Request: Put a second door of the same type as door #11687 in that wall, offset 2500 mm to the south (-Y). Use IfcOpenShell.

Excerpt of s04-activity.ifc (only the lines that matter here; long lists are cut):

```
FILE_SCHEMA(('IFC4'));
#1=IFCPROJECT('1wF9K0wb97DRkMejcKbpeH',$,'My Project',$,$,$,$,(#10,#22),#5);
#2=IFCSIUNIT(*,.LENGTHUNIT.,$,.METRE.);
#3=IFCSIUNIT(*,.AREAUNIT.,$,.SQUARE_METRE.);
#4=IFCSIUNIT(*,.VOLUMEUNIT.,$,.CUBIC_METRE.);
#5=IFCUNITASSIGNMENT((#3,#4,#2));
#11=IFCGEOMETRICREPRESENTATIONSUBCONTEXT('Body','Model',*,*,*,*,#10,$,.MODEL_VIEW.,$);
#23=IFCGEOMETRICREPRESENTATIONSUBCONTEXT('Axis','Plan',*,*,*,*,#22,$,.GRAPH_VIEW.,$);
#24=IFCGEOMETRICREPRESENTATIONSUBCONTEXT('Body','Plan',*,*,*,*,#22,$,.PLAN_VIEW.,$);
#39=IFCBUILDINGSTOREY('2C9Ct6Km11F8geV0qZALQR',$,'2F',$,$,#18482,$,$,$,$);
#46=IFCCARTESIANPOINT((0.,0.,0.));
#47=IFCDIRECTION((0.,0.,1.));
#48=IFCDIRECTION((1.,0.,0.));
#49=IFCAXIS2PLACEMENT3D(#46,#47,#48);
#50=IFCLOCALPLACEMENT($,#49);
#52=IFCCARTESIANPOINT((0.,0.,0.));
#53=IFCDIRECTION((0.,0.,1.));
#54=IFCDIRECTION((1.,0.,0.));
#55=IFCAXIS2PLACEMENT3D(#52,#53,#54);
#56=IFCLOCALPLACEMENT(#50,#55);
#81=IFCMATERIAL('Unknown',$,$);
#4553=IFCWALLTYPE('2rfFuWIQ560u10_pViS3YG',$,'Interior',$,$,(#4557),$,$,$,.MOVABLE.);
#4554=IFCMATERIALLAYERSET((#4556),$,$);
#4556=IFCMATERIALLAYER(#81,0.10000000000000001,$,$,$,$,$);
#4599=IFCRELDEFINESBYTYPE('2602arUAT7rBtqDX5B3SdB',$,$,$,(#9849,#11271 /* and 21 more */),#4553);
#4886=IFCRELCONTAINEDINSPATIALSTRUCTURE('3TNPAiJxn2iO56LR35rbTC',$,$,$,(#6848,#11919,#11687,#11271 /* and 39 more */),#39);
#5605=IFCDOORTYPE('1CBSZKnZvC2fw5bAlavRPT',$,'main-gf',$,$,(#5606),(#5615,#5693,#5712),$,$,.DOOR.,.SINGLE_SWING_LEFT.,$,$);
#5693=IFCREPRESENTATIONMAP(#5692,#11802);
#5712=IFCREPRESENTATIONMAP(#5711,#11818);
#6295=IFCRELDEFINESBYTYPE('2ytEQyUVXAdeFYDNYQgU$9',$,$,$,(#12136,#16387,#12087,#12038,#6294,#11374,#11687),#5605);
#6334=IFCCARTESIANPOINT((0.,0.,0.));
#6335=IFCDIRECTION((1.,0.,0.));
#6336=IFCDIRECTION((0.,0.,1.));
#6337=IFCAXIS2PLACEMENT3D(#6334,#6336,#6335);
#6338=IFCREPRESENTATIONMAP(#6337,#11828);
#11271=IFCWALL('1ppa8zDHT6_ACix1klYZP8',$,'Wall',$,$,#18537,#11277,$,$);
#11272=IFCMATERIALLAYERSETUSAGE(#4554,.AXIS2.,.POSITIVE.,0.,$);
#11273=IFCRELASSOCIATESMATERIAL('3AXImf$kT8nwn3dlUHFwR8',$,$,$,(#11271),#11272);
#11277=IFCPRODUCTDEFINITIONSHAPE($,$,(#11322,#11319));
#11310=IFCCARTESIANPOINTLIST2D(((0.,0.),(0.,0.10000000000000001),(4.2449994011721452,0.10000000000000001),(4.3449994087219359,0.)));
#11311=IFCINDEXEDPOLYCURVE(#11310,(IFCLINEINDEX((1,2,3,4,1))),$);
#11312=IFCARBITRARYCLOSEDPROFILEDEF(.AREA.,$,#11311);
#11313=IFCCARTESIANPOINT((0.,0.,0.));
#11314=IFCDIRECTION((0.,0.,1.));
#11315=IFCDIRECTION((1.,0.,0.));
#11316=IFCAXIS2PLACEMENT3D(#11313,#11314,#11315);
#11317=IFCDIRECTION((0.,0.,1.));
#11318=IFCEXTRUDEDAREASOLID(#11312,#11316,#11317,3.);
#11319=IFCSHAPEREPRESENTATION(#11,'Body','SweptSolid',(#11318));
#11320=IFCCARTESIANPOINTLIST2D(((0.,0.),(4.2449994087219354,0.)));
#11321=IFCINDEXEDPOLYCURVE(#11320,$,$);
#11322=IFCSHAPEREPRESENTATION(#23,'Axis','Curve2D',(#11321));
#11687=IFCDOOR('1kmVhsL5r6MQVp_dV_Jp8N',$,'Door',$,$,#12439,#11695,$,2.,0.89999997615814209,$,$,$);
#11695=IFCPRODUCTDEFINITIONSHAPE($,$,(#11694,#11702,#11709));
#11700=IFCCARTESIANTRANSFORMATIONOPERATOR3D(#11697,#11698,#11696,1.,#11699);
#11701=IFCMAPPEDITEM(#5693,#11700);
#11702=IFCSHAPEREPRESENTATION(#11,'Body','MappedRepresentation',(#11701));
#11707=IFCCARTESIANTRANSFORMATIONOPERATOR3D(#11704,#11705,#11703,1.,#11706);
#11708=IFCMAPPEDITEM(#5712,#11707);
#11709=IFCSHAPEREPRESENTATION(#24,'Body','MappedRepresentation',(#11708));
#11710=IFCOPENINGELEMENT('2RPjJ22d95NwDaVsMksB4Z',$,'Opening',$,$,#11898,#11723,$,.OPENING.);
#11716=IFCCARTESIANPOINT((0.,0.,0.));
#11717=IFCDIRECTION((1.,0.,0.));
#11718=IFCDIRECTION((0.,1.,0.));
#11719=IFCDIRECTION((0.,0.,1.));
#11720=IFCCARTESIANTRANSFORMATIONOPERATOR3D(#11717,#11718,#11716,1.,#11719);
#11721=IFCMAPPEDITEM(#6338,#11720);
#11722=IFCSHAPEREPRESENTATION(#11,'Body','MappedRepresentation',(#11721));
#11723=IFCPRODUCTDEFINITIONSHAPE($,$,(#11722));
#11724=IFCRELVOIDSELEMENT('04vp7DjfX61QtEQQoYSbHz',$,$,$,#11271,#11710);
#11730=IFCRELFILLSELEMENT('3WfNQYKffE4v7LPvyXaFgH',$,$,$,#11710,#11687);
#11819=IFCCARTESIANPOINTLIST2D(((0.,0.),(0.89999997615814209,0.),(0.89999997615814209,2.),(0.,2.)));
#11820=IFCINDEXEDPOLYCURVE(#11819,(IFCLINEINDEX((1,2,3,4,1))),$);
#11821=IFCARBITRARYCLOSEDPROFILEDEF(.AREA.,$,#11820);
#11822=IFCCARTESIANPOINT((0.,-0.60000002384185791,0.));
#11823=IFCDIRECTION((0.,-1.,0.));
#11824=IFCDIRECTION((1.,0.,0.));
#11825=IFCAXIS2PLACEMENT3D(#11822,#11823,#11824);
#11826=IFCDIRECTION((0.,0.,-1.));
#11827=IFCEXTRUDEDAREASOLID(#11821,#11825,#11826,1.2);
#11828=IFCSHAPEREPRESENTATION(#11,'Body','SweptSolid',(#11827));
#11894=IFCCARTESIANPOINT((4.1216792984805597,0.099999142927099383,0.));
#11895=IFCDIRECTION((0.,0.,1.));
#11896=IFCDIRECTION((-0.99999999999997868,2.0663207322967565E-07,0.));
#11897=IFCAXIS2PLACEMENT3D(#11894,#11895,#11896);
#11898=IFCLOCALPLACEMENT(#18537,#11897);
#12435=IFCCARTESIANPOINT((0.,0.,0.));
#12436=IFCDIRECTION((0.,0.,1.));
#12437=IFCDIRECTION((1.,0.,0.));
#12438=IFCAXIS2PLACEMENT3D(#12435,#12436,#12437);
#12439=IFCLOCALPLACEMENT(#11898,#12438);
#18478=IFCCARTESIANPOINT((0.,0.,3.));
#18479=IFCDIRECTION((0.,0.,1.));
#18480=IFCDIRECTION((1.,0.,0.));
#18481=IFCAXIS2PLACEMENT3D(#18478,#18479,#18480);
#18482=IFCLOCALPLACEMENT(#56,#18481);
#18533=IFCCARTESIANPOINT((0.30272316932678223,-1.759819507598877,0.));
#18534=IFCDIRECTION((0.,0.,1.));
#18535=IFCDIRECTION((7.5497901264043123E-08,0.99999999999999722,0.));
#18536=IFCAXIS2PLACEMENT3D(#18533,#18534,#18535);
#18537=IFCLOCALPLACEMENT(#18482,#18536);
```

```python
import ifcopenshell
import ifcopenshell.api.feature
import ifcopenshell.api.geometry
import ifcopenshell.api.root
import ifcopenshell.geom
import ifcopenshell.util.element
import ifcopenshell.util.placement
import ifcopenshell.util.shape
import ifcopenshell.util.unit

model = ifcopenshell.open("s04-activity.ifc")
unit_scale = ifcopenshell.util.unit.calculate_unit_scale(model)
settings = ifcopenshell.geom.settings()


def volume(element):
    """Net volume in cubic metres, openings subtracted."""
    shape = ifcopenshell.geom.create_shape(settings, element)
    return ifcopenshell.util.shape.get_volume(shape.geometry)


door = model.by_guid("1kmVhsL5r6MQVp_dV_Jp8N")
opening = door.FillsVoids[0].RelatingOpeningElement
wall = opening.VoidsElements[0].RelatingBuildingElement
before = volume(wall)
shift = ifcopenshell.util.placement.get_local_placement(wall.ObjectPlacement)[:3, 0] * -2.5 / unit_scale

# copy_class copies the void relationship, type, container and properties, but no geometry.
new_opening = ifcopenshell.api.root.copy_class(model, product=opening)
new_opening.Representation = ifcopenshell.util.element.copy_deep(
    model, opening.Representation, exclude=["IfcGeometricRepresentationContext", "IfcRepresentationMap"]
)
new_door = ifcopenshell.api.root.copy_class(model, product=door)
new_door.Representation = ifcopenshell.util.element.copy_deep(
    model, door.Representation, exclude=["IfcGeometricRepresentationContext", "IfcRepresentationMap"]
)
ifcopenshell.api.feature.add_filling(model, opening=new_opening, element=new_door)

for old, new in ((opening, new_opening), (door, new_door)):
    matrix = ifcopenshell.util.placement.get_local_placement(old.ObjectPlacement)
    matrix[:3, 3] += shift
    ifcopenshell.api.geometry.edit_object_placement(model, product=new, matrix=matrix, is_si=False)

after = volume(wall)

print(f"wall volume {before:.3f} -> {after:.3f} m3")

model.write("s04-activity-out.ifc")
```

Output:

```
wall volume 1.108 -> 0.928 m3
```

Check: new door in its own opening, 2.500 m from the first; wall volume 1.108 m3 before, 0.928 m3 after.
